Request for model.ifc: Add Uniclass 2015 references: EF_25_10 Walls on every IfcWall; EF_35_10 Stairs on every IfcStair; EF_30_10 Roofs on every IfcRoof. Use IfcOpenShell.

First a look at what the model holds.

```python
import ifcopenshell

model = ifcopenshell.open("model.ifc")
print(model.schema)
print("classifications:", [c.Name for c in model.by_type("IfcClassification")])
for ifc_class in ("IfcDoor", "IfcRoof", "IfcStair", "IfcWall", "IfcWindow"):
    print(ifc_class, len(model.by_type(ifc_class)))
```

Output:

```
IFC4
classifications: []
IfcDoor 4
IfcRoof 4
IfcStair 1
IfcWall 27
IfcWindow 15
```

```python
import ifcopenshell
import ifcopenshell.api.classification

model = ifcopenshell.open("model.ifc")

system = ifcopenshell.api.classification.add_classification(model, classification="Uniclass 2015")

codes = {
    "IfcWall": ("EF_25_10", "Walls"),
    "IfcStair": ("EF_35_10", "Stairs"),
    "IfcRoof": ("EF_30_10", "Roofs"),
}
for ifc_class, (code, name) in codes.items():
    products = model.by_type(ifc_class)
    ifcopenshell.api.classification.add_reference(
        model, products=products, classification=system, identification=code, name=name
    )
    print(code, len(products))

model.write("model-out.ifc")
```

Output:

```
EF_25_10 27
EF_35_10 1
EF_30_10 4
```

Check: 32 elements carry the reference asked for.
